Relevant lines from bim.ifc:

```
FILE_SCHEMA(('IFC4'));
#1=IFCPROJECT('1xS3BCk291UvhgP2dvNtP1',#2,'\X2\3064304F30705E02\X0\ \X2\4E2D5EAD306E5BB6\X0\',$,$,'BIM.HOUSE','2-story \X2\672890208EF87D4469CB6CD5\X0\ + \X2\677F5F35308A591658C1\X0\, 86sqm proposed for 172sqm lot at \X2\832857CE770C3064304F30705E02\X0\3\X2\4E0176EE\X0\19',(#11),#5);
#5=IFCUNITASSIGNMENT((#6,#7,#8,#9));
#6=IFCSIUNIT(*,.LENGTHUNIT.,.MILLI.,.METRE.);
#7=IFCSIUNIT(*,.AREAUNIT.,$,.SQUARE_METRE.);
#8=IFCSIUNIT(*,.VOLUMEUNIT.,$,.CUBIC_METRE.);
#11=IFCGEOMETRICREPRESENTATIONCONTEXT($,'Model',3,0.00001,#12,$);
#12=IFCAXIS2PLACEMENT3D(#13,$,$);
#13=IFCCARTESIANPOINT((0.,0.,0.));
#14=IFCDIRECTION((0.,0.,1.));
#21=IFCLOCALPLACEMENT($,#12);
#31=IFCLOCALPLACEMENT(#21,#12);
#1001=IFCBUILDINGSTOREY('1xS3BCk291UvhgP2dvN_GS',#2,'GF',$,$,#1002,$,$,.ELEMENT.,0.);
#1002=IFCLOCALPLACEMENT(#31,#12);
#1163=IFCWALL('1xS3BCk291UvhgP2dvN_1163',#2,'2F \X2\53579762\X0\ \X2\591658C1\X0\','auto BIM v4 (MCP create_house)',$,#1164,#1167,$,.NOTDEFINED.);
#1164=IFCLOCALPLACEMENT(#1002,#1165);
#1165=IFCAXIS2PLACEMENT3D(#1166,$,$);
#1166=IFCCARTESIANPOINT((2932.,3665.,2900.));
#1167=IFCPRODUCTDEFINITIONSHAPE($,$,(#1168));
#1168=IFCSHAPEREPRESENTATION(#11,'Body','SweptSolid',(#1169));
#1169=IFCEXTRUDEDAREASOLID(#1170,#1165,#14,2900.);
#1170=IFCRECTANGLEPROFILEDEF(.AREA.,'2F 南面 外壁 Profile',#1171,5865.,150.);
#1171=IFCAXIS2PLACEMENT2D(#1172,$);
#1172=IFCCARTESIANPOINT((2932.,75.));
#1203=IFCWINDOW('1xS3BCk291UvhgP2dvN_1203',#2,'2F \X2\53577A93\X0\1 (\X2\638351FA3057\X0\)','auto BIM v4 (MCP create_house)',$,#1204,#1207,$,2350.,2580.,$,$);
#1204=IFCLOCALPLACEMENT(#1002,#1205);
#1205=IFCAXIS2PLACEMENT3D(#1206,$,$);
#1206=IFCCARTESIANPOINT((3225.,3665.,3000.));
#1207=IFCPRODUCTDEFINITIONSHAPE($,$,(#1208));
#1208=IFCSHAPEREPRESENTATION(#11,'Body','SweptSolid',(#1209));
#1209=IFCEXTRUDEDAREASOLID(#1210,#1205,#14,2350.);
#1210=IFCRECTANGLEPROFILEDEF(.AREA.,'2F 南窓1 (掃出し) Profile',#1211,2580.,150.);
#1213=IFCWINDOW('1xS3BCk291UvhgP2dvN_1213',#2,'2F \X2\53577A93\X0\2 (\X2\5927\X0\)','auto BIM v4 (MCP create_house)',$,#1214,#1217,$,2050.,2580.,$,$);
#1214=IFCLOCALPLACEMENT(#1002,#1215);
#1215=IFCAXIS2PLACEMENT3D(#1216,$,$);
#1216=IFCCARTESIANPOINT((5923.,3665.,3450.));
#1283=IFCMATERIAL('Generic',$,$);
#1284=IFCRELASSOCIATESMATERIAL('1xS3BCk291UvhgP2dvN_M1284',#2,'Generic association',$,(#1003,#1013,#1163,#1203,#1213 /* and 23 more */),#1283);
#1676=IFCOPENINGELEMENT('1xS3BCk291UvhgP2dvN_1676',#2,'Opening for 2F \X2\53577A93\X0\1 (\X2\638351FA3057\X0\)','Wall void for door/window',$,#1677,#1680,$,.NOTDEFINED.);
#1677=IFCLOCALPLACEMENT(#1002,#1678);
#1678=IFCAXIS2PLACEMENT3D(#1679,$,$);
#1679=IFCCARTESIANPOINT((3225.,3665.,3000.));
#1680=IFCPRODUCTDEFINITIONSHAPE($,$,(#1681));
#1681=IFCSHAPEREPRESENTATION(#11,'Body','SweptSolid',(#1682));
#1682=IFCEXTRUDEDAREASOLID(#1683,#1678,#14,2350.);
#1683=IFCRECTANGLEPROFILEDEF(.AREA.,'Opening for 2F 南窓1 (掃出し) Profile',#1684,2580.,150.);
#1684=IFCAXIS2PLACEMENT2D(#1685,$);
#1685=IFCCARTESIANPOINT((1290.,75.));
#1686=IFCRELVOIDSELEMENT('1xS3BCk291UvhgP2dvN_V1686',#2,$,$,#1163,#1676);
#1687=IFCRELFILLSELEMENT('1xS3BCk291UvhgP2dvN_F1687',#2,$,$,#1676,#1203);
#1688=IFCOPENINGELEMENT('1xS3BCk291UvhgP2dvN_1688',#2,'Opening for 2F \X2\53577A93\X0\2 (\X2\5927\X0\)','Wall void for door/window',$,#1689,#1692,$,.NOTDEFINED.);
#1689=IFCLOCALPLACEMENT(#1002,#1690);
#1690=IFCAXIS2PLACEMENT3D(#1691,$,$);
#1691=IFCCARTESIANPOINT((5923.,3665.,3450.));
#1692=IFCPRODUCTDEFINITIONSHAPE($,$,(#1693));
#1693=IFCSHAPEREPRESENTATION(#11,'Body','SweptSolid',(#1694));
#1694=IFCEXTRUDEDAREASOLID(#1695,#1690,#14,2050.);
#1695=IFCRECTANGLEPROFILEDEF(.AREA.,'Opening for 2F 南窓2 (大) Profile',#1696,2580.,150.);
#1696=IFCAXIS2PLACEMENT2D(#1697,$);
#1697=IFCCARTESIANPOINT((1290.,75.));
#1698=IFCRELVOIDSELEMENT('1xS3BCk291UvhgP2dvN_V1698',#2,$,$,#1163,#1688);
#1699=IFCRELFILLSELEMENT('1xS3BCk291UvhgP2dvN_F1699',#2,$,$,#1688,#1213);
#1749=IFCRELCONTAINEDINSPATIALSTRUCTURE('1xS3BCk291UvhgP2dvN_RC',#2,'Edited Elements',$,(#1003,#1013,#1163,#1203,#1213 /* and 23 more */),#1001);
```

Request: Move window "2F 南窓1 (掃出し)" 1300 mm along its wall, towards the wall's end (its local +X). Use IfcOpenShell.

```python
import ifcopenshell
import ifcopenshell.api.geometry
import ifcopenshell.util.placement
import ifcopenshell.util.unit

model = ifcopenshell.open("bim.ifc")
unit_scale = ifcopenshell.util.unit.calculate_unit_scale(model)

window = model.by_guid("1xS3BCk291UvhgP2dvN_1203")
opening = window.FillsVoids[0].RelatingOpeningElement
wall = opening.VoidsElements[0].RelatingBuildingElement

wall_matrix = ifcopenshell.util.placement.get_local_placement(wall.ObjectPlacement)
shift = wall_matrix[:3, 0] * 1.3 / unit_scale
before = ifcopenshell.util.placement.get_local_placement(window.ObjectPlacement)[:3, 3].copy()

# The window is not placed relative to its opening, so move both.
for product in (opening, window):
    matrix = ifcopenshell.util.placement.get_local_placement(product.ObjectPlacement)
    matrix[:3, 3] += shift
    ifcopenshell.api.geometry.edit_object_placement(model, product=product, matrix=matrix, is_si=False)

after = ifcopenshell.util.placement.get_local_placement(window.ObjectPlacement)[:3, 3]
print("window moved by", (after - before).round(3) + 0.0)

model.write("bim_updated.ifc")
```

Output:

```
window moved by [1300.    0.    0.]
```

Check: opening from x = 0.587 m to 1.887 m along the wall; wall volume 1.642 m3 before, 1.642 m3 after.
